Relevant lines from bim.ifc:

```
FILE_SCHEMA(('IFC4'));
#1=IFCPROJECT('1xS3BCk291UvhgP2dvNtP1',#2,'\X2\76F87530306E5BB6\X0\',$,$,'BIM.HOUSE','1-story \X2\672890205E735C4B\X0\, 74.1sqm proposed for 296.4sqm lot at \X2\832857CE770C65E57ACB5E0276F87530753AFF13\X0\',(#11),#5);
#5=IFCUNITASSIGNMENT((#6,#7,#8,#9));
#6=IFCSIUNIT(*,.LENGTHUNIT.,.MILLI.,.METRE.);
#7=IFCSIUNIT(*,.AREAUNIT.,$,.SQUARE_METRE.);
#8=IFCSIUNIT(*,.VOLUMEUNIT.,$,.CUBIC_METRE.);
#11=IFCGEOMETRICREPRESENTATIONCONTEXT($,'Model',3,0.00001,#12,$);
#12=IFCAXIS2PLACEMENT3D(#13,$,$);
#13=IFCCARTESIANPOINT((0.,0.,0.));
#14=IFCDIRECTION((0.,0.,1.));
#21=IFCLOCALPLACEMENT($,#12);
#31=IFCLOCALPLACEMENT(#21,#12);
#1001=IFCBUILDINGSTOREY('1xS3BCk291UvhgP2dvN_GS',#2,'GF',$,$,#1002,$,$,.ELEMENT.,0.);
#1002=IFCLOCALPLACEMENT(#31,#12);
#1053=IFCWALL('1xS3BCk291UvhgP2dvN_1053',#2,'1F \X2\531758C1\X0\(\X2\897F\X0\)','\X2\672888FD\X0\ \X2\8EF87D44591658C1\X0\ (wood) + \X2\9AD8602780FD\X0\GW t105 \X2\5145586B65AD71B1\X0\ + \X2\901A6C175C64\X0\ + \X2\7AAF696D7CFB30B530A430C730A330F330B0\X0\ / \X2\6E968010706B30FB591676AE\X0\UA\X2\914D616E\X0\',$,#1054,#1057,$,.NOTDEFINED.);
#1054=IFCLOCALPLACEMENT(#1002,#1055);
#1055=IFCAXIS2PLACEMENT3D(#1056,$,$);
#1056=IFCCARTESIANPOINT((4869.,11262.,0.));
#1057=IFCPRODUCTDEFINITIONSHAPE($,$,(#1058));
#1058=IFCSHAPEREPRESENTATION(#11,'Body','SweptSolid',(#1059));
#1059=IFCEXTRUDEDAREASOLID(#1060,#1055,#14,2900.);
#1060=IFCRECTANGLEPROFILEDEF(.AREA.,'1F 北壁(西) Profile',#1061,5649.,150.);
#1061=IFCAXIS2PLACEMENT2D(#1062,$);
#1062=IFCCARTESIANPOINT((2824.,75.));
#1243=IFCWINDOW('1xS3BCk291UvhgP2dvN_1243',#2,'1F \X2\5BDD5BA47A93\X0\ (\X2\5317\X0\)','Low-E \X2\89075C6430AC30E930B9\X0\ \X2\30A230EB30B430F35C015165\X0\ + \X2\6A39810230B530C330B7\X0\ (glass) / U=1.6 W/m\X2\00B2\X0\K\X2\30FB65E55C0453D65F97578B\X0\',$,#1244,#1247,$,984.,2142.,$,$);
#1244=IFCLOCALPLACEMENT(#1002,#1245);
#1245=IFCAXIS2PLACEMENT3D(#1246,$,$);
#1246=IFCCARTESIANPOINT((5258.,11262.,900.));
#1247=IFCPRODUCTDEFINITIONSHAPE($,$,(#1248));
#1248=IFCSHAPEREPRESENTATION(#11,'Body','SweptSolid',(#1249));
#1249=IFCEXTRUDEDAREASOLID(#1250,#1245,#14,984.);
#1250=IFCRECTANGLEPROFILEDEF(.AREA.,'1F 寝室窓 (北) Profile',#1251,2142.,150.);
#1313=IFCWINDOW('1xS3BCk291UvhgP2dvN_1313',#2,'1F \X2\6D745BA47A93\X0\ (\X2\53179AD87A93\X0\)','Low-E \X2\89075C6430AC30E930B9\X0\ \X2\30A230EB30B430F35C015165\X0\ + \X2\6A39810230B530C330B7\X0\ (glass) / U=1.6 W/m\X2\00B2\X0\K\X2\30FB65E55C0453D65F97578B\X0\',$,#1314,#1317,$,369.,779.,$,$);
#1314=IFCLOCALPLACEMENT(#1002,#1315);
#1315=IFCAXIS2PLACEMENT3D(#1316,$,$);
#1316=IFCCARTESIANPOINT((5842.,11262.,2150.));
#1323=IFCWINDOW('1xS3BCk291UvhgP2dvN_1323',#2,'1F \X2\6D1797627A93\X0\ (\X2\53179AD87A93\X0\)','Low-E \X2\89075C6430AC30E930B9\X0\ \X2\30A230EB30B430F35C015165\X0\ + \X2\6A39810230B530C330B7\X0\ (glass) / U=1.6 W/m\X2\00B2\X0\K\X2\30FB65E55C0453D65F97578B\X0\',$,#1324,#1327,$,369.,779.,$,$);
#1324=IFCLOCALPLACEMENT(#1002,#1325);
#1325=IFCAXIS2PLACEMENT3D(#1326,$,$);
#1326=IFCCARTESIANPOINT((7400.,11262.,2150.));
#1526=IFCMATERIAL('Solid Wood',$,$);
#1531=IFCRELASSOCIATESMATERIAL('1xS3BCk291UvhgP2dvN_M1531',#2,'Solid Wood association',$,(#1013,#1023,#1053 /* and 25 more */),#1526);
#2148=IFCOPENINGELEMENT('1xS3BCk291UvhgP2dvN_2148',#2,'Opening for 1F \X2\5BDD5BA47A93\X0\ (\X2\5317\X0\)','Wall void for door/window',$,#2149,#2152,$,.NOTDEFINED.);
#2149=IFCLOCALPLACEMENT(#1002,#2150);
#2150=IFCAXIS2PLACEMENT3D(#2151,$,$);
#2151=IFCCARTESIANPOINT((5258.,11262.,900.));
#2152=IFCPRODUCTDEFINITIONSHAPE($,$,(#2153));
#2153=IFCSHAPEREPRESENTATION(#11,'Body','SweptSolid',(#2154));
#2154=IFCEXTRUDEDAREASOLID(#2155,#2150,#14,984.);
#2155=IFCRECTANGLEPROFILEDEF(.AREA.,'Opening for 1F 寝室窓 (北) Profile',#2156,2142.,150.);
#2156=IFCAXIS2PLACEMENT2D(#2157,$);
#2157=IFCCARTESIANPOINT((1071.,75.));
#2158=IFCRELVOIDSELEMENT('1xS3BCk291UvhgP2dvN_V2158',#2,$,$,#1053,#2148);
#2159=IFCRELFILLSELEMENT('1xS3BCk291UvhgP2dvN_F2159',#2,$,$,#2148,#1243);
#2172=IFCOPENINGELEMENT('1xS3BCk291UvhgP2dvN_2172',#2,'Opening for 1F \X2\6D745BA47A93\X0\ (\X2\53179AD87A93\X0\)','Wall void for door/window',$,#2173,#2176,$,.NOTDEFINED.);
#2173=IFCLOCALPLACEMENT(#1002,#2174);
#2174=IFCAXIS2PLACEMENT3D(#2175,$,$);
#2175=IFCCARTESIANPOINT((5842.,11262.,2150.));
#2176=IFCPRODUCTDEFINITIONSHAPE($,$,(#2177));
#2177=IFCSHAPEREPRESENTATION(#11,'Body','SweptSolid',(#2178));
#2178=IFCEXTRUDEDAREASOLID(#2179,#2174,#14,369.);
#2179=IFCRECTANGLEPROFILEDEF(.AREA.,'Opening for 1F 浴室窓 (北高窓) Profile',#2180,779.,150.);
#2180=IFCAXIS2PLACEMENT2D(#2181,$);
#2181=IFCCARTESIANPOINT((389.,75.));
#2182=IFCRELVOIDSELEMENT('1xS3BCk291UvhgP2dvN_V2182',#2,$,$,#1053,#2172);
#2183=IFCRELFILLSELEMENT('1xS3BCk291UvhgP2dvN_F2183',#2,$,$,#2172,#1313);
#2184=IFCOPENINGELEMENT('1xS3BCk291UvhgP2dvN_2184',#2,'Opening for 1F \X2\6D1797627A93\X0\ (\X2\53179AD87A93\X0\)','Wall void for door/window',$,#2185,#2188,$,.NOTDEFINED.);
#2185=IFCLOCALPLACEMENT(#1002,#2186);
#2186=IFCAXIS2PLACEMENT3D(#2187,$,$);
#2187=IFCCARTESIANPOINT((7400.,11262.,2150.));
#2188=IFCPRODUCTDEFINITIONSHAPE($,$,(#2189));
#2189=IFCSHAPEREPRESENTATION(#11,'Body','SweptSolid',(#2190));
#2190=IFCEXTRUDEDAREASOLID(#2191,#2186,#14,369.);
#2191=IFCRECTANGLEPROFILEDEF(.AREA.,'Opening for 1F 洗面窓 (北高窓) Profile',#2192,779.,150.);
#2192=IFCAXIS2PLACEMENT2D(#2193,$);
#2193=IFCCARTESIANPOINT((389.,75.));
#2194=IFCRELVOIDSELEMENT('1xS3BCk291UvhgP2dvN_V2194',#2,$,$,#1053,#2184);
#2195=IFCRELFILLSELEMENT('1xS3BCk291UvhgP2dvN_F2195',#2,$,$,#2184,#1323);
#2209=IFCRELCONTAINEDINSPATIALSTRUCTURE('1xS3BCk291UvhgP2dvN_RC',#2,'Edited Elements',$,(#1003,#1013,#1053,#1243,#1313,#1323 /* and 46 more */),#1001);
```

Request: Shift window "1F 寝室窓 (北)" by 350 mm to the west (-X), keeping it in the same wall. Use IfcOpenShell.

```python
import ifcopenshell
import ifcopenshell.api.geometry
import ifcopenshell.util.placement
import ifcopenshell.util.unit

model = ifcopenshell.open("bim.ifc")
unit_scale = ifcopenshell.util.unit.calculate_unit_scale(model)

window = model.by_guid("1xS3BCk291UvhgP2dvN_1243")
opening = window.FillsVoids[0].RelatingOpeningElement
wall = opening.VoidsElements[0].RelatingBuildingElement

wall_matrix = ifcopenshell.util.placement.get_local_placement(wall.ObjectPlacement)
shift = wall_matrix[:3, 0] * -0.35 / unit_scale
before = ifcopenshell.util.placement.get_local_placement(window.ObjectPlacement)[:3, 3].copy()

# The window is not placed relative to its opening, so move both.
for product in (opening, window):
    matrix = ifcopenshell.util.placement.get_local_placement(product.ObjectPlacement)
    matrix[:3, 3] += shift
    ifcopenshell.api.geometry.edit_object_placement(model, product=product, matrix=matrix, is_si=False)

after = ifcopenshell.util.placement.get_local_placement(window.ObjectPlacement)[:3, 3]
print("window moved by", (after - before).round(3) + 0.0)

model.write("bim_v2.ifc")
```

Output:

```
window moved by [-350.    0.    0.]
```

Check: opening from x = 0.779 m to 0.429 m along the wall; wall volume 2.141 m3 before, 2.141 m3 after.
